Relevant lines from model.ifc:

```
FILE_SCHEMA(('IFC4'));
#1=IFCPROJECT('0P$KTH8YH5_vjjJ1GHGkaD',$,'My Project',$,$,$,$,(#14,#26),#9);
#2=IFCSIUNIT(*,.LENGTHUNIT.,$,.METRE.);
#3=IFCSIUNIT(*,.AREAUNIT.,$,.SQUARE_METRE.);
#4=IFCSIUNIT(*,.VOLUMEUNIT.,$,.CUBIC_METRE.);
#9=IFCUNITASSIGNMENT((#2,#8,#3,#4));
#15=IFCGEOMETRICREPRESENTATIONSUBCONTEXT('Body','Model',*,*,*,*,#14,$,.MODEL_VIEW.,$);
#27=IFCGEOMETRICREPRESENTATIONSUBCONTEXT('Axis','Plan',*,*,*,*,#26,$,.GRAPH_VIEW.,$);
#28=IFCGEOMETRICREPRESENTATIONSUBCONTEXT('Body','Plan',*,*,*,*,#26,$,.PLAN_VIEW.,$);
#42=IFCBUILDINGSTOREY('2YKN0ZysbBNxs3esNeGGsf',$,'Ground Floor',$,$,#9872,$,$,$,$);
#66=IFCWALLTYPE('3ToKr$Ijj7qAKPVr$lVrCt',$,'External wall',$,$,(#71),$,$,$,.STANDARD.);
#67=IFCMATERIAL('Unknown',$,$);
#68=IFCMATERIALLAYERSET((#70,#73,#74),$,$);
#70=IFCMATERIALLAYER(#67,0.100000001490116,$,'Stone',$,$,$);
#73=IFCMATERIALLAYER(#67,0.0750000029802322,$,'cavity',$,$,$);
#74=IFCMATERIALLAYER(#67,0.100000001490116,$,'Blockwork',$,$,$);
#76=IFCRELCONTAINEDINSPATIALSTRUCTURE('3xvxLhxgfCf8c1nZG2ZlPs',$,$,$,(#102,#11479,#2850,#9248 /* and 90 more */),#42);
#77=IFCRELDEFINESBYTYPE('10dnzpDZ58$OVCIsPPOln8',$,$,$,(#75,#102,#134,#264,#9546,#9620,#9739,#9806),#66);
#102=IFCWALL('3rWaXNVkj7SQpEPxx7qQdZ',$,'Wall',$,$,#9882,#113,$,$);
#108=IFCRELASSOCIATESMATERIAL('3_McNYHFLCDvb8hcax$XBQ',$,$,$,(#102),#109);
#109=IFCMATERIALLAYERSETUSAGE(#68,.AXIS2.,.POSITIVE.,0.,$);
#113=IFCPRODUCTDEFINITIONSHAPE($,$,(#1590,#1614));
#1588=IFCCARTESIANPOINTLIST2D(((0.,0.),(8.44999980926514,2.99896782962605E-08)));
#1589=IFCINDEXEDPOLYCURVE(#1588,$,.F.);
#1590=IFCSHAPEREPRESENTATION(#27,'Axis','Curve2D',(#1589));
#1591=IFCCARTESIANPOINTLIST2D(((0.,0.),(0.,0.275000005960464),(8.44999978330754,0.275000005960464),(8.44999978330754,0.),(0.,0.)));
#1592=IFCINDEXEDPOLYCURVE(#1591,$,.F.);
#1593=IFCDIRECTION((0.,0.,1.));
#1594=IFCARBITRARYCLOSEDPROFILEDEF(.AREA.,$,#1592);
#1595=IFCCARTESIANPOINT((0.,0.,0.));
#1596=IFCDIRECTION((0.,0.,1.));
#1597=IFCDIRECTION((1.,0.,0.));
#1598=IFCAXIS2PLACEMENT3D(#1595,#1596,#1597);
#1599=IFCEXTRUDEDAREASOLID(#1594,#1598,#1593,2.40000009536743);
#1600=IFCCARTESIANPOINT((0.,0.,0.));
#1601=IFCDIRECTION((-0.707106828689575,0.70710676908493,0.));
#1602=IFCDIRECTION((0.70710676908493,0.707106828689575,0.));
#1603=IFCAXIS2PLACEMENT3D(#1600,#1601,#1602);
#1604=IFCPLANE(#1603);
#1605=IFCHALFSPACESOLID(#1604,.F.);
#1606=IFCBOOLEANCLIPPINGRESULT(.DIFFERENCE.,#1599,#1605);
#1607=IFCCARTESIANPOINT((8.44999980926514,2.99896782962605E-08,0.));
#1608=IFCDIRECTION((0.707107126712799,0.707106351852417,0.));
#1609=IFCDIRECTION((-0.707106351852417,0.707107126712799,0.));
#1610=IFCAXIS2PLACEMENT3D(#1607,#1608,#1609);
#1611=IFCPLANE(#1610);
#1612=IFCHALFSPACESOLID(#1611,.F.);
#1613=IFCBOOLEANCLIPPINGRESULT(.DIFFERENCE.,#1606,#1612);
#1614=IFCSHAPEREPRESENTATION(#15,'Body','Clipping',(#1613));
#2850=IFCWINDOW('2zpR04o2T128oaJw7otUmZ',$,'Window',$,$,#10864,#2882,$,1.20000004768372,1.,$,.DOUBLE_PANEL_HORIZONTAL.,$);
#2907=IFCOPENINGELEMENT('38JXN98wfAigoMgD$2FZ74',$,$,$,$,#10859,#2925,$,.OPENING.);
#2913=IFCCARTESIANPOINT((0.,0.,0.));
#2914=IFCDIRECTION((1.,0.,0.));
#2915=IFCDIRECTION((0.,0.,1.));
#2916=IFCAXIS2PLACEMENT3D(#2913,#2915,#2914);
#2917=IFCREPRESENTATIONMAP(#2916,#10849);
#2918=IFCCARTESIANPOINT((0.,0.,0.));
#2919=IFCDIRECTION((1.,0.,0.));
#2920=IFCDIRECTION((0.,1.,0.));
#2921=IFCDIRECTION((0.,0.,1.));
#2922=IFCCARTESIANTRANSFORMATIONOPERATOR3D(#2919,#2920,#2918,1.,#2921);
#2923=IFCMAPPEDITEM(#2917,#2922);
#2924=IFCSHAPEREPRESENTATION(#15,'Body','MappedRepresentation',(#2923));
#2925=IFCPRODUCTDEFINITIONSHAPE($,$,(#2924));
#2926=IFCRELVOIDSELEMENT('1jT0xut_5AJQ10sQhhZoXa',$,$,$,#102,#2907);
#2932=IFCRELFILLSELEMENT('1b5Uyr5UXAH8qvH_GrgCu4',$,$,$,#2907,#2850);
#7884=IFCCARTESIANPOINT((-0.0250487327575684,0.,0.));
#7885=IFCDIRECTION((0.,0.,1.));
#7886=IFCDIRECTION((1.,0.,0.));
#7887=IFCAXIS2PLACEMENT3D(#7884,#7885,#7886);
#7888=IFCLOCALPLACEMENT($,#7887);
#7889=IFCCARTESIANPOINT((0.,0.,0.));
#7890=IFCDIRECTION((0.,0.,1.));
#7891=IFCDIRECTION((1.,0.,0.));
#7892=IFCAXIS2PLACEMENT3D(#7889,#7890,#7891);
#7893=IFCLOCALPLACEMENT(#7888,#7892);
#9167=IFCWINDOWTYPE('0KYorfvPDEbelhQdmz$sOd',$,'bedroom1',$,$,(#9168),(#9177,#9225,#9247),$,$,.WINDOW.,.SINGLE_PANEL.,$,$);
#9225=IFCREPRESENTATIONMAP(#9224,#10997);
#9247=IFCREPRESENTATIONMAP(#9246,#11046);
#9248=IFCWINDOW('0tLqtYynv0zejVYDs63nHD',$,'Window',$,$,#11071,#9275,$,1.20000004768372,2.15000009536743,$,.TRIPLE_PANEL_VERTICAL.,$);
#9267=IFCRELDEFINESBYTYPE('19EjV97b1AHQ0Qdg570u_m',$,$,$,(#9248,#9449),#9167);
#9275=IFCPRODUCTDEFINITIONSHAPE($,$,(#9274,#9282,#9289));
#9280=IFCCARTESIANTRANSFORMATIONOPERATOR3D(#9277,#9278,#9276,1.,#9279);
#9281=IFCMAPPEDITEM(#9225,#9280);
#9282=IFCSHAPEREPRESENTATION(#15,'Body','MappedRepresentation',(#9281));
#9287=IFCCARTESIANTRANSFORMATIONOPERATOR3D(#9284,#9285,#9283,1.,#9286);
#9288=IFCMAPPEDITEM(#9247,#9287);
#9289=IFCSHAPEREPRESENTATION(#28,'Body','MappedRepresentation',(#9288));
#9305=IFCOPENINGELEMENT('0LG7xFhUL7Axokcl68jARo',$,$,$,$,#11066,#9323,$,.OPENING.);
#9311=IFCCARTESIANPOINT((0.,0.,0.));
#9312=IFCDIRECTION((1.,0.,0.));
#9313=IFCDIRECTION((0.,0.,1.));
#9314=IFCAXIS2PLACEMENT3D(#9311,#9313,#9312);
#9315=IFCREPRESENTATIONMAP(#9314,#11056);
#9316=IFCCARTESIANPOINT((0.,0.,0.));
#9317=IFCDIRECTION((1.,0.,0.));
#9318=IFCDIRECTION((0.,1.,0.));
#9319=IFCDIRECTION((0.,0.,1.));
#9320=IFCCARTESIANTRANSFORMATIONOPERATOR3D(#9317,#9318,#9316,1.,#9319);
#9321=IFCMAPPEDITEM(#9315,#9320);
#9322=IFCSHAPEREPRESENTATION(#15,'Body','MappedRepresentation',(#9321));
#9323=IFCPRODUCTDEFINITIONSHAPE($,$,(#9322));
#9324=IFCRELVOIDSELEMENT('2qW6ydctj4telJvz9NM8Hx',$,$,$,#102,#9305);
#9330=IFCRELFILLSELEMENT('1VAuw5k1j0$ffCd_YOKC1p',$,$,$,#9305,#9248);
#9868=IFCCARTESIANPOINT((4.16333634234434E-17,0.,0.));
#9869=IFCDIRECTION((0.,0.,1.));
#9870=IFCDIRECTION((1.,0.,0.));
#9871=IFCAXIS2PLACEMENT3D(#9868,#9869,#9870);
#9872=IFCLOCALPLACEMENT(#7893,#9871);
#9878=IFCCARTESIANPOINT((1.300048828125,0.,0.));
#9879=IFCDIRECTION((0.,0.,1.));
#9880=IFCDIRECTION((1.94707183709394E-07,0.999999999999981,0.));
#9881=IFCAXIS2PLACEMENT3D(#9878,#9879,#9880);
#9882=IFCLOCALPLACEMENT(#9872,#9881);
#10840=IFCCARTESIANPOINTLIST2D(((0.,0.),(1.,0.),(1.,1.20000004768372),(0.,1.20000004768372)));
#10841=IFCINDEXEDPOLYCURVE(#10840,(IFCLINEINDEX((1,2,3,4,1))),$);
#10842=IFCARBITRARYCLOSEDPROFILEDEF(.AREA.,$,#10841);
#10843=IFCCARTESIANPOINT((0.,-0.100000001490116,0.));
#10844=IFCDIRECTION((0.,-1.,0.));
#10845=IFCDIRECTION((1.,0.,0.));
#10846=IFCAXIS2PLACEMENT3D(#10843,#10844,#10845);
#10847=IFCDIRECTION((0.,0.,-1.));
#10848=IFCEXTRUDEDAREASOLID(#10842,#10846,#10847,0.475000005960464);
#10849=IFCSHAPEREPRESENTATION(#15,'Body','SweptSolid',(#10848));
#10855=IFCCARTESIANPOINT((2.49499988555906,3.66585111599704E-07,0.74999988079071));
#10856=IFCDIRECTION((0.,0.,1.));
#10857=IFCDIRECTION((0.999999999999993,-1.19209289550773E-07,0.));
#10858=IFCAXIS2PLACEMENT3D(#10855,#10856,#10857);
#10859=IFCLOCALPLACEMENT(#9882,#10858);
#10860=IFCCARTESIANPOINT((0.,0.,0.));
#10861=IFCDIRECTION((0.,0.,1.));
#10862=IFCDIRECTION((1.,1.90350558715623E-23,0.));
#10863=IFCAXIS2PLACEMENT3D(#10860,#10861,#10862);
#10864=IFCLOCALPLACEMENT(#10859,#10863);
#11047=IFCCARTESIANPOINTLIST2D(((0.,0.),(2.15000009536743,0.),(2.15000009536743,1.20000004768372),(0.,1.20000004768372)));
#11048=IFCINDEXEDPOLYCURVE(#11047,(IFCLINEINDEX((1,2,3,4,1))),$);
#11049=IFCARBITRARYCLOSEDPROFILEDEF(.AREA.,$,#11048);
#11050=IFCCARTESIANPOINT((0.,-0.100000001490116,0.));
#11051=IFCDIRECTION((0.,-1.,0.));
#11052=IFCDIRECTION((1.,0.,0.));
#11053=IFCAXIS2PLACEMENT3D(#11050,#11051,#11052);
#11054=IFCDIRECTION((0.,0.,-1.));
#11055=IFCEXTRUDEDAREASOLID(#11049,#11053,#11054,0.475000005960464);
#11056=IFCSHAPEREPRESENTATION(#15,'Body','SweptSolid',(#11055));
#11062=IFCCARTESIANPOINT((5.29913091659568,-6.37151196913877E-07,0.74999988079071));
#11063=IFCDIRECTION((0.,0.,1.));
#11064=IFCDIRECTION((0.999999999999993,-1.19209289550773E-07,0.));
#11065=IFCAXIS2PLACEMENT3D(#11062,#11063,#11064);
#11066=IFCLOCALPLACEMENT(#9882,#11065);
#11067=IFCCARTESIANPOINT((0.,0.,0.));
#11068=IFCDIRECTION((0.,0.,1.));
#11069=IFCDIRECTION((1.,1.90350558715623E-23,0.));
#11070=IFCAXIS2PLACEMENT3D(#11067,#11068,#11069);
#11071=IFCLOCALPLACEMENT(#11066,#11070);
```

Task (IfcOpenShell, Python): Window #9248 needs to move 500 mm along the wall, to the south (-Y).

```python
import ifcopenshell
import ifcopenshell.api.geometry
import ifcopenshell.util.placement
import ifcopenshell.util.unit

model = ifcopenshell.open("model.ifc")
unit_scale = ifcopenshell.util.unit.calculate_unit_scale(model)

window = model.by_id(9248)
opening = window.FillsVoids[0].RelatingOpeningElement
wall = opening.VoidsElements[0].RelatingBuildingElement

wall_matrix = ifcopenshell.util.placement.get_local_placement(wall.ObjectPlacement)
shift = wall_matrix[:3, 0] * -0.5 / unit_scale
before = ifcopenshell.util.placement.get_local_placement(window.ObjectPlacement)[:3, 3].copy()

# The window is placed relative to its opening, so it follows when the opening moves.
matrix = ifcopenshell.util.placement.get_local_placement(opening.ObjectPlacement)
matrix[:3, 3] += shift
ifcopenshell.api.geometry.edit_object_placement(
    model, product=opening, matrix=matrix, is_si=False, should_transform_children=True
)

after = ifcopenshell.util.placement.get_local_placement(window.ObjectPlacement)[:3, 3]
print("window moved by", (after - before).round(3) + 0.0)

model.write("model_v2.ifc")
```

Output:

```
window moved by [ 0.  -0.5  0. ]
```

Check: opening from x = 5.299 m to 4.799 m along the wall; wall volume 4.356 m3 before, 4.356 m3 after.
